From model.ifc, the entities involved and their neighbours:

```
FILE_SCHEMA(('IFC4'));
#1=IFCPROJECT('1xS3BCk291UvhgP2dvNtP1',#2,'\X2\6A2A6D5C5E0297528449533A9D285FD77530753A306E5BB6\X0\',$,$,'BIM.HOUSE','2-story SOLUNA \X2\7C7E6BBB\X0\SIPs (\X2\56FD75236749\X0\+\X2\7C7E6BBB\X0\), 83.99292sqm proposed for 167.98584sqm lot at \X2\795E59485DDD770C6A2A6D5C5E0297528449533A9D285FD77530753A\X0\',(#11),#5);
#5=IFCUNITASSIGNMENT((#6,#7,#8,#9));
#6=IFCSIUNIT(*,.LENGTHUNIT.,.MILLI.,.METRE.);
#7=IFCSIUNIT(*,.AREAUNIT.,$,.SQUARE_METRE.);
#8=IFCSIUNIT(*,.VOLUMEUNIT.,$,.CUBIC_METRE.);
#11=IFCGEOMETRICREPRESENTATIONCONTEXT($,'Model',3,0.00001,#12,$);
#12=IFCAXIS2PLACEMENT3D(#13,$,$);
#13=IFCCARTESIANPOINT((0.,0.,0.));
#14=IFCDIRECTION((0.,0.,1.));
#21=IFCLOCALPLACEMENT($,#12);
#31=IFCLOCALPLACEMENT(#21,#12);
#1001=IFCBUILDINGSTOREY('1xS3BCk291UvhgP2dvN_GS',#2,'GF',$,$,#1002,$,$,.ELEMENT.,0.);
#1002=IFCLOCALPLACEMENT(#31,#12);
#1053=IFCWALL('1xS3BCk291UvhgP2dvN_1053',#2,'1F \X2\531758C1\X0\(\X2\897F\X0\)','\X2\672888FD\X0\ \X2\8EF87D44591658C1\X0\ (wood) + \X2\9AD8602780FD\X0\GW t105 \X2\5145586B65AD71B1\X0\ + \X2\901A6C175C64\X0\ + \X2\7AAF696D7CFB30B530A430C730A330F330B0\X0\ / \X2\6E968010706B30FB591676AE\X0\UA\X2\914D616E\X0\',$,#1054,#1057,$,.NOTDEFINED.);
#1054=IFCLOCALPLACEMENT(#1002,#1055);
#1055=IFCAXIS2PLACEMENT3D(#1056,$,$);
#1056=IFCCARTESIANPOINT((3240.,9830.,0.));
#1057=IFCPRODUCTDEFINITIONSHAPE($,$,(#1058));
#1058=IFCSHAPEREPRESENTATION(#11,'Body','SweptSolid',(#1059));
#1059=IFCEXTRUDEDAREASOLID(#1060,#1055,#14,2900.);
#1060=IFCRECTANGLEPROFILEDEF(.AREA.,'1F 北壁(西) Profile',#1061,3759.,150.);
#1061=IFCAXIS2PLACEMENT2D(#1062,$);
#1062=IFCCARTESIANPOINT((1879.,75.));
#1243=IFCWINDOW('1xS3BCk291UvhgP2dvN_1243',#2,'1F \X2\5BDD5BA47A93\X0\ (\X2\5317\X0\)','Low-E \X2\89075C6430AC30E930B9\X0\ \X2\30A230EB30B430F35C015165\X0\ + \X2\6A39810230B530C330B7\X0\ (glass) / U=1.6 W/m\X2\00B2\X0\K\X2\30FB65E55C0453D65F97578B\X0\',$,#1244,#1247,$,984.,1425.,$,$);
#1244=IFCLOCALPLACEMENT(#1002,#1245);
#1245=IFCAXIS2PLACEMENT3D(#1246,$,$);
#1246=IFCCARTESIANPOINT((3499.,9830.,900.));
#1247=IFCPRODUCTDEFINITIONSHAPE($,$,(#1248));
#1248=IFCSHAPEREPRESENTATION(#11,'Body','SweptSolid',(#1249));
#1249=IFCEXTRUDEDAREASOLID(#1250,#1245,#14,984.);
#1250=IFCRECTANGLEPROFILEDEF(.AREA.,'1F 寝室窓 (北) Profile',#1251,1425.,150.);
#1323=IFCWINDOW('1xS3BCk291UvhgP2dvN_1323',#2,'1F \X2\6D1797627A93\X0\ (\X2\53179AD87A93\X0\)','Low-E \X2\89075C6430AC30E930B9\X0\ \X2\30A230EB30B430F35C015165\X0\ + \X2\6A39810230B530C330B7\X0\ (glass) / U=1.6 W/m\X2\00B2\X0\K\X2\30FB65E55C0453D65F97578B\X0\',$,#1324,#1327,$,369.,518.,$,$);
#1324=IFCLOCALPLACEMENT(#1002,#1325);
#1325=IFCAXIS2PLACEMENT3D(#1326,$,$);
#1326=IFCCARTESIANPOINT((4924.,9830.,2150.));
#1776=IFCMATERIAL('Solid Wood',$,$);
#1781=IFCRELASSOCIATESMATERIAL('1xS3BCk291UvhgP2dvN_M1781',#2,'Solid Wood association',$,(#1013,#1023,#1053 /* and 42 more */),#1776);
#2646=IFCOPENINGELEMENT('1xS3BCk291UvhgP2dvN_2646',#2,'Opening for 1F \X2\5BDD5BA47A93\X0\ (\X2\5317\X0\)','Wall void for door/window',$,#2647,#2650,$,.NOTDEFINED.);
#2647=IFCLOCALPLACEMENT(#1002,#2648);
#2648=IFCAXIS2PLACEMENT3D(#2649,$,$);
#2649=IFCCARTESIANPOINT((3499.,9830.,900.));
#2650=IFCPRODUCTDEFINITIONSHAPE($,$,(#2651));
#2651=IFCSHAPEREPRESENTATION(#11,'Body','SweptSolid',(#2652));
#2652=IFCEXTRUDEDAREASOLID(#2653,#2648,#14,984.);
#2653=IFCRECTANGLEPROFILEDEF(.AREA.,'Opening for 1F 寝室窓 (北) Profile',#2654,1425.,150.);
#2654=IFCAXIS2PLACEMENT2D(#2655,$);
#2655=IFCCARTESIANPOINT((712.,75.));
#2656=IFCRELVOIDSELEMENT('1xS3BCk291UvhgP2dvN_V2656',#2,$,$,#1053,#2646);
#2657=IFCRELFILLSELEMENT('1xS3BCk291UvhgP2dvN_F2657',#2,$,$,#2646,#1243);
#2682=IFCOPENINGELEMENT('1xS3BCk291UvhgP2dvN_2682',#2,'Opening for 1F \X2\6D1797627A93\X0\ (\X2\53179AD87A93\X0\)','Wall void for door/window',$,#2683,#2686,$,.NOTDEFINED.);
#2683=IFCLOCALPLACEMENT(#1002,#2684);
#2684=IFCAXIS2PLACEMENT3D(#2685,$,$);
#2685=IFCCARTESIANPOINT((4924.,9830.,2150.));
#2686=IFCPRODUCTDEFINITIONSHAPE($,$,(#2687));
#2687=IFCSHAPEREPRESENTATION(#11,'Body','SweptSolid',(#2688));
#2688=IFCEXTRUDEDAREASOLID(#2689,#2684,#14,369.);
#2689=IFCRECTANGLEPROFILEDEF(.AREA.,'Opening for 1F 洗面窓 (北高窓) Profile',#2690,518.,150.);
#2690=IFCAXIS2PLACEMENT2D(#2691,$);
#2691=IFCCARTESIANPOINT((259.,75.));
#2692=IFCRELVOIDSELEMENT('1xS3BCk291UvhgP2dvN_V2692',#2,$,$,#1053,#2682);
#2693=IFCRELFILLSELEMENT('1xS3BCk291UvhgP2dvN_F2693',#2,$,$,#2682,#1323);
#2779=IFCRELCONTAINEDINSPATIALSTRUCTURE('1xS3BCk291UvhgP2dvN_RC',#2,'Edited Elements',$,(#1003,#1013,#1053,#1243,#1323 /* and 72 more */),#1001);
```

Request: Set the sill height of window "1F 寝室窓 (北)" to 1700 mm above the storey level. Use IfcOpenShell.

```python
import numpy as np
import ifcopenshell
import ifcopenshell.api.geometry
import ifcopenshell.geom
import ifcopenshell.util.element
import ifcopenshell.util.placement
import ifcopenshell.util.shape
import ifcopenshell.util.unit

model = ifcopenshell.open("model.ifc")
unit_scale = ifcopenshell.util.unit.calculate_unit_scale(model)

window = model.by_guid("1xS3BCk291UvhgP2dvN_1243")
opening = window.FillsVoids[0].RelatingOpeningElement
storey = ifcopenshell.util.element.get_container(window, ifc_class="IfcBuildingStorey")
level = ifcopenshell.util.placement.get_local_placement(storey.ObjectPlacement)[2, 3]

# The opening's origin need not be at the sill, so measure its lowest point.
shape = ifcopenshell.geom.create_shape(ifcopenshell.geom.settings(), opening)
bottom = ifcopenshell.util.shape.get_shape_bottom_elevation(shape, shape.geometry) / unit_scale
dz = level + 1.7 / unit_scale - bottom

shift = np.array([0.0, 0.0, dz])
# The window is not placed relative to its opening, so move both.
for product in (opening, window):
    matrix = ifcopenshell.util.placement.get_local_placement(product.ObjectPlacement)
    matrix[:3, 3] += shift
    ifcopenshell.api.geometry.edit_object_placement(model, product=product, matrix=matrix, is_si=False)

print(f"moved by {dz * unit_scale:+.3f} m")

model.write("model-out.ifc")
```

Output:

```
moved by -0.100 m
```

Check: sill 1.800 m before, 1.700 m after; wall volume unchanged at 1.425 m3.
